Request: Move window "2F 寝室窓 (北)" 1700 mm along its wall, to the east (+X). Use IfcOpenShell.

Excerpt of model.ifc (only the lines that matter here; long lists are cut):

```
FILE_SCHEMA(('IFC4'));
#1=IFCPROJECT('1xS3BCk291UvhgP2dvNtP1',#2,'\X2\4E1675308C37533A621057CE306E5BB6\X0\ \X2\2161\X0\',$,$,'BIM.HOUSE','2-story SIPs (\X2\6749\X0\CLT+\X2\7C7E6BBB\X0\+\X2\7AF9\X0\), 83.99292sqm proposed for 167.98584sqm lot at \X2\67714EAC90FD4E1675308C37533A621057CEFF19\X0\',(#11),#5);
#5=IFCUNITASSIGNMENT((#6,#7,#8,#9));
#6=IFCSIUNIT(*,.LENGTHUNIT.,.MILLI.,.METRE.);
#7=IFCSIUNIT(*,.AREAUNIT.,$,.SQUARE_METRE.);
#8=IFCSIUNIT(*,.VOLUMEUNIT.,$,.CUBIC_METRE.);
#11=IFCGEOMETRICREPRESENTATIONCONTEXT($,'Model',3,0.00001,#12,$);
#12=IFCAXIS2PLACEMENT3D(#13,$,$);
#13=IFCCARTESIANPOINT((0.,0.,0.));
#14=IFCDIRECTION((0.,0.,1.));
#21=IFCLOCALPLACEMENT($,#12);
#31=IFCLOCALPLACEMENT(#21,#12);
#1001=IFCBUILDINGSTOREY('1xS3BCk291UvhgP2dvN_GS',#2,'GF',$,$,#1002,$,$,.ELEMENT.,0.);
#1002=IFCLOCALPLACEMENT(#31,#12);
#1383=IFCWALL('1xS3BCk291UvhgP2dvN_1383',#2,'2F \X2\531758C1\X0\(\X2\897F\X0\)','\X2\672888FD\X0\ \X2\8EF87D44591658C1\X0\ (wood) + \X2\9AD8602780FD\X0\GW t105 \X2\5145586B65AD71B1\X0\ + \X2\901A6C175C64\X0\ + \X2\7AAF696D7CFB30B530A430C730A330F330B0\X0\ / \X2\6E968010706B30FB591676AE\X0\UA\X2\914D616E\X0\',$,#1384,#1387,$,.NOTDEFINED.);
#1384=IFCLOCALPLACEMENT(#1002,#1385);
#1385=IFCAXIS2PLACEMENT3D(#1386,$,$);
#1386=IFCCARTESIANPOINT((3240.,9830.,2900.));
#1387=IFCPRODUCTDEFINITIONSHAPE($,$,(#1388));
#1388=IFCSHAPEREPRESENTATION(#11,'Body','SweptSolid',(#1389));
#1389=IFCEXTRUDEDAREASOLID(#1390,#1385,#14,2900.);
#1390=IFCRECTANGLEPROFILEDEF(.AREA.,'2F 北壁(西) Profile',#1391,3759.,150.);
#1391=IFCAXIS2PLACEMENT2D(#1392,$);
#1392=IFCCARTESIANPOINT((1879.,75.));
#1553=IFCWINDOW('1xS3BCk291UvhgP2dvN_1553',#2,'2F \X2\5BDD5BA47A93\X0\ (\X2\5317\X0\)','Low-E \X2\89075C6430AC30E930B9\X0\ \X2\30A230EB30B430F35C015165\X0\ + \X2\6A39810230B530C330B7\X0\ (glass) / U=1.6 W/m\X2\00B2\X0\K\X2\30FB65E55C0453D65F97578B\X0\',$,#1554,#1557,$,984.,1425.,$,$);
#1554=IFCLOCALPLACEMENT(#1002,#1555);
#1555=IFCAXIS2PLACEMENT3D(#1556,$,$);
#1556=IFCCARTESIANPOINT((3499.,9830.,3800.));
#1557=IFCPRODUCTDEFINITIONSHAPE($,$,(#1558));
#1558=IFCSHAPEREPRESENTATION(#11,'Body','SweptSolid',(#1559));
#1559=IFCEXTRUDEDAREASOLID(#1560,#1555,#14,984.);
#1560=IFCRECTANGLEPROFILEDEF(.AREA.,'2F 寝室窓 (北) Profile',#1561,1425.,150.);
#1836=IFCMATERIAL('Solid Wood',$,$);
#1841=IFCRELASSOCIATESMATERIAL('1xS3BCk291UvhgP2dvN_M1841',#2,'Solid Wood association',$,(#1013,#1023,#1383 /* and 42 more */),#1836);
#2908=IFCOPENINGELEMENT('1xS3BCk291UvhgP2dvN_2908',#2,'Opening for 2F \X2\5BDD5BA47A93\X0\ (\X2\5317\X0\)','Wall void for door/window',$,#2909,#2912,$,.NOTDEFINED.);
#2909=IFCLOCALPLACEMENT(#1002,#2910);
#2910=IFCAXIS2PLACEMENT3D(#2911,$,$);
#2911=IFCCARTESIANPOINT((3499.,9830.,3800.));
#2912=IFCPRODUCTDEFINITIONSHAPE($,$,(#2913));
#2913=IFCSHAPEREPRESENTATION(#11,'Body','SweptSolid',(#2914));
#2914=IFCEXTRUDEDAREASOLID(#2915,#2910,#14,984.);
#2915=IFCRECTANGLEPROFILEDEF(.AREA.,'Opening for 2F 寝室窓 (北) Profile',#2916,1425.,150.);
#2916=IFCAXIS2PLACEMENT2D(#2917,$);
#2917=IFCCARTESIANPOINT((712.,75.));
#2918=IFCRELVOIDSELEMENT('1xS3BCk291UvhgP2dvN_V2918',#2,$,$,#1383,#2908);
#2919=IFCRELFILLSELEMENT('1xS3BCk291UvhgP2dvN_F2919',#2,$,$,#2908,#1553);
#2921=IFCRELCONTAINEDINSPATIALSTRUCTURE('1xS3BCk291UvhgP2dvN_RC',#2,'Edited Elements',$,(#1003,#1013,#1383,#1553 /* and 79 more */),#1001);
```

```python
import ifcopenshell
import ifcopenshell.api.geometry
import ifcopenshell.util.placement
import ifcopenshell.util.unit

model = ifcopenshell.open("model.ifc")
unit_scale = ifcopenshell.util.unit.calculate_unit_scale(model)

window = model.by_guid("1xS3BCk291UvhgP2dvN_1553")
opening = window.FillsVoids[0].RelatingOpeningElement
wall = opening.VoidsElements[0].RelatingBuildingElement

wall_matrix = ifcopenshell.util.placement.get_local_placement(wall.ObjectPlacement)
shift = wall_matrix[:3, 0] * 1.7 / unit_scale
before = ifcopenshell.util.placement.get_local_placement(window.ObjectPlacement)[:3, 3].copy()

# The window is not placed relative to its opening, so move both.
for product in (opening, window):
    matrix = ifcopenshell.util.placement.get_local_placement(product.ObjectPlacement)
    matrix[:3, 3] += shift
    ifcopenshell.api.geometry.edit_object_placement(model, product=product, matrix=matrix, is_si=False)

after = ifcopenshell.util.placement.get_local_placement(window.ObjectPlacement)[:3, 3]
print("window moved by", (after - before).round(3) + 0.0)

model.write("model_edited.ifc")
```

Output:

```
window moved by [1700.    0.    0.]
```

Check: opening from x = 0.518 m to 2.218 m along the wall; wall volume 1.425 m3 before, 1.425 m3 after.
